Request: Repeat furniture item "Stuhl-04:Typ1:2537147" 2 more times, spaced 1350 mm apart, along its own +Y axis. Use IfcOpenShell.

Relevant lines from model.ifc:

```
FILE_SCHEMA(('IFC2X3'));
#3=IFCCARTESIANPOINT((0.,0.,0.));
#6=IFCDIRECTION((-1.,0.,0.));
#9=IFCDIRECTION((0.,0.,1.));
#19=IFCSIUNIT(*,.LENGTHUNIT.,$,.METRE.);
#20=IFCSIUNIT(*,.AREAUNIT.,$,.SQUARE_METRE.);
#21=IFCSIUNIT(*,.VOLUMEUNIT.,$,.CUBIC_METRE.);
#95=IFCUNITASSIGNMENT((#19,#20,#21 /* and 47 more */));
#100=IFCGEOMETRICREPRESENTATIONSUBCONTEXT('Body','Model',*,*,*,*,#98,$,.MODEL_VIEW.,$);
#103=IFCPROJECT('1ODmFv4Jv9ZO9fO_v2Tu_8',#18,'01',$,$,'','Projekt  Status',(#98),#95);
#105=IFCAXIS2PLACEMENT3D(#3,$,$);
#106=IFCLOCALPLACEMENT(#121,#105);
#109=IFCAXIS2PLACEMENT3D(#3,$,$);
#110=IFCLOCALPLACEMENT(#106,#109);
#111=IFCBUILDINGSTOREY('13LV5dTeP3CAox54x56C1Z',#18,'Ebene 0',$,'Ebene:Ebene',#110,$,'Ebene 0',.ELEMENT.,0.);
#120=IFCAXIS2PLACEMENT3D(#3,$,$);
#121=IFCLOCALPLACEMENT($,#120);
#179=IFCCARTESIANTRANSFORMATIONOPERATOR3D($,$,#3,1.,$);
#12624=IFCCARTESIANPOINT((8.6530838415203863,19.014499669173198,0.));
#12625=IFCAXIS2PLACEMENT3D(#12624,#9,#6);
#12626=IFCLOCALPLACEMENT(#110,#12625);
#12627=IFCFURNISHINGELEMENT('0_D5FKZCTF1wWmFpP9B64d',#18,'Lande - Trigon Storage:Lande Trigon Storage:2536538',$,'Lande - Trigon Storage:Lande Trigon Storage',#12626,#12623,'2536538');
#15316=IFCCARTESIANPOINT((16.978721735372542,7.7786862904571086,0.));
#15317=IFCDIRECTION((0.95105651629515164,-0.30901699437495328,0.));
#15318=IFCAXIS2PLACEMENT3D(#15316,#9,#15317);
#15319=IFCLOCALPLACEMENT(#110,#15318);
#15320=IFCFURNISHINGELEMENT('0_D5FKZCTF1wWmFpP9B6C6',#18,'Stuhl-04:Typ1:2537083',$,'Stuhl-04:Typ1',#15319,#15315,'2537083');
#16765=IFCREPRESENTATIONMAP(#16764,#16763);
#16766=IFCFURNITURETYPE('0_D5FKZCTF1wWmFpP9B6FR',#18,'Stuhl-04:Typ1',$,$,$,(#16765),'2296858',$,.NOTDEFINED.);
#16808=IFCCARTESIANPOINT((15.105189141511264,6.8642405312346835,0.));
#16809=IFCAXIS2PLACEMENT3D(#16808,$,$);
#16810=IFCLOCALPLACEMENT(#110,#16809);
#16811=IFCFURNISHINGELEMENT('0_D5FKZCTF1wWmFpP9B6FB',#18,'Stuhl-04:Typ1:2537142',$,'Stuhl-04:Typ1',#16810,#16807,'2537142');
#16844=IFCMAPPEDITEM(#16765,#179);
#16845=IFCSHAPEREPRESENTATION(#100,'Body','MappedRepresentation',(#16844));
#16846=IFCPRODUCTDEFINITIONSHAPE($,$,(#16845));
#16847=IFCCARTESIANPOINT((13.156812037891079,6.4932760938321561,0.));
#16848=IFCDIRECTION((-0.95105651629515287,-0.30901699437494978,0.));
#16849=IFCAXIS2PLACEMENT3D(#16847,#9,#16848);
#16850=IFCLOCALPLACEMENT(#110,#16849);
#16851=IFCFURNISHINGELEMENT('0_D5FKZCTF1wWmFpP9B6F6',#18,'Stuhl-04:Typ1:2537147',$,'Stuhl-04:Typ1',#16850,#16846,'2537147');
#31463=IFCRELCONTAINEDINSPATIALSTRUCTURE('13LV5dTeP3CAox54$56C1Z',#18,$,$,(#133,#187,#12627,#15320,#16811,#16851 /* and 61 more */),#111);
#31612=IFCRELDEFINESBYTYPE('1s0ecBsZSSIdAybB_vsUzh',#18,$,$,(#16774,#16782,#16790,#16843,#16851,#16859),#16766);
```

```python
import ifcopenshell
import ifcopenshell.api.geometry
import ifcopenshell.api.root
import ifcopenshell.util.element
import ifcopenshell.util.placement

model = ifcopenshell.open("model.ifc")

source = model.by_guid("0_D5FKZCTF1wWmFpP9B6F6")
base = ifcopenshell.util.placement.get_local_placement(source.ObjectPlacement)
step = base[:3, 1] * 1.35

for i in range(1, 3):
    copy = ifcopenshell.api.root.copy_class(model, product=source)
    copy.Representation = ifcopenshell.util.element.copy_deep(
        model, source.Representation, exclude=["IfcGeometricRepresentationContext", "IfcRepresentationMap"]
    )
    copy.Name = "Stuhl-04:Typ1"
    copy.Tag = None
    matrix = base.copy()
    matrix[:3, 3] += i * step
    print("added at", matrix[:3, 3].round(3) + 0.0)
    ifcopenshell.api.geometry.edit_object_placement(model, product=copy, matrix=matrix, is_si=False)

model.write("model-out.ifc")
```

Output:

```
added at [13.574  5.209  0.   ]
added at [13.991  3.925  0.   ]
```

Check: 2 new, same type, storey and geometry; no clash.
